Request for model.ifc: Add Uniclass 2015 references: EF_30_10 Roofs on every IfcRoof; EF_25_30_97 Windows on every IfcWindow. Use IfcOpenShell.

First a look at what the model holds.

```python
import ifcopenshell

model = ifcopenshell.open("model.ifc")
print(model.schema)
print("classifications:", [c.Name for c in model.by_type("IfcClassification")])
for ifc_class in ("IfcDoor", "IfcRoof", "IfcStair", "IfcWall", "IfcWindow"):
    print(ifc_class, len(model.by_type(ifc_class)))
```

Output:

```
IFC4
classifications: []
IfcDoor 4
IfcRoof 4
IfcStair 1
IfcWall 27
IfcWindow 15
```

```python
import ifcopenshell
import ifcopenshell.api.classification

model = ifcopenshell.open("model.ifc")

system = ifcopenshell.api.classification.add_classification(model, classification="Uniclass 2015")

codes = {
    "IfcRoof": ("EF_30_10", "Roofs"),
    "IfcWindow": ("EF_25_30_97", "Windows"),
}
for ifc_class, (code, name) in codes.items():
    products = model.by_type(ifc_class)
    ifcopenshell.api.classification.add_reference(
        model, products=products, classification=system, identification=code, name=name
    )
    print(code, len(products))

model.write("model_v2.ifc")
```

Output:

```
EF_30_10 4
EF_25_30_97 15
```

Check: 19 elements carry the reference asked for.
